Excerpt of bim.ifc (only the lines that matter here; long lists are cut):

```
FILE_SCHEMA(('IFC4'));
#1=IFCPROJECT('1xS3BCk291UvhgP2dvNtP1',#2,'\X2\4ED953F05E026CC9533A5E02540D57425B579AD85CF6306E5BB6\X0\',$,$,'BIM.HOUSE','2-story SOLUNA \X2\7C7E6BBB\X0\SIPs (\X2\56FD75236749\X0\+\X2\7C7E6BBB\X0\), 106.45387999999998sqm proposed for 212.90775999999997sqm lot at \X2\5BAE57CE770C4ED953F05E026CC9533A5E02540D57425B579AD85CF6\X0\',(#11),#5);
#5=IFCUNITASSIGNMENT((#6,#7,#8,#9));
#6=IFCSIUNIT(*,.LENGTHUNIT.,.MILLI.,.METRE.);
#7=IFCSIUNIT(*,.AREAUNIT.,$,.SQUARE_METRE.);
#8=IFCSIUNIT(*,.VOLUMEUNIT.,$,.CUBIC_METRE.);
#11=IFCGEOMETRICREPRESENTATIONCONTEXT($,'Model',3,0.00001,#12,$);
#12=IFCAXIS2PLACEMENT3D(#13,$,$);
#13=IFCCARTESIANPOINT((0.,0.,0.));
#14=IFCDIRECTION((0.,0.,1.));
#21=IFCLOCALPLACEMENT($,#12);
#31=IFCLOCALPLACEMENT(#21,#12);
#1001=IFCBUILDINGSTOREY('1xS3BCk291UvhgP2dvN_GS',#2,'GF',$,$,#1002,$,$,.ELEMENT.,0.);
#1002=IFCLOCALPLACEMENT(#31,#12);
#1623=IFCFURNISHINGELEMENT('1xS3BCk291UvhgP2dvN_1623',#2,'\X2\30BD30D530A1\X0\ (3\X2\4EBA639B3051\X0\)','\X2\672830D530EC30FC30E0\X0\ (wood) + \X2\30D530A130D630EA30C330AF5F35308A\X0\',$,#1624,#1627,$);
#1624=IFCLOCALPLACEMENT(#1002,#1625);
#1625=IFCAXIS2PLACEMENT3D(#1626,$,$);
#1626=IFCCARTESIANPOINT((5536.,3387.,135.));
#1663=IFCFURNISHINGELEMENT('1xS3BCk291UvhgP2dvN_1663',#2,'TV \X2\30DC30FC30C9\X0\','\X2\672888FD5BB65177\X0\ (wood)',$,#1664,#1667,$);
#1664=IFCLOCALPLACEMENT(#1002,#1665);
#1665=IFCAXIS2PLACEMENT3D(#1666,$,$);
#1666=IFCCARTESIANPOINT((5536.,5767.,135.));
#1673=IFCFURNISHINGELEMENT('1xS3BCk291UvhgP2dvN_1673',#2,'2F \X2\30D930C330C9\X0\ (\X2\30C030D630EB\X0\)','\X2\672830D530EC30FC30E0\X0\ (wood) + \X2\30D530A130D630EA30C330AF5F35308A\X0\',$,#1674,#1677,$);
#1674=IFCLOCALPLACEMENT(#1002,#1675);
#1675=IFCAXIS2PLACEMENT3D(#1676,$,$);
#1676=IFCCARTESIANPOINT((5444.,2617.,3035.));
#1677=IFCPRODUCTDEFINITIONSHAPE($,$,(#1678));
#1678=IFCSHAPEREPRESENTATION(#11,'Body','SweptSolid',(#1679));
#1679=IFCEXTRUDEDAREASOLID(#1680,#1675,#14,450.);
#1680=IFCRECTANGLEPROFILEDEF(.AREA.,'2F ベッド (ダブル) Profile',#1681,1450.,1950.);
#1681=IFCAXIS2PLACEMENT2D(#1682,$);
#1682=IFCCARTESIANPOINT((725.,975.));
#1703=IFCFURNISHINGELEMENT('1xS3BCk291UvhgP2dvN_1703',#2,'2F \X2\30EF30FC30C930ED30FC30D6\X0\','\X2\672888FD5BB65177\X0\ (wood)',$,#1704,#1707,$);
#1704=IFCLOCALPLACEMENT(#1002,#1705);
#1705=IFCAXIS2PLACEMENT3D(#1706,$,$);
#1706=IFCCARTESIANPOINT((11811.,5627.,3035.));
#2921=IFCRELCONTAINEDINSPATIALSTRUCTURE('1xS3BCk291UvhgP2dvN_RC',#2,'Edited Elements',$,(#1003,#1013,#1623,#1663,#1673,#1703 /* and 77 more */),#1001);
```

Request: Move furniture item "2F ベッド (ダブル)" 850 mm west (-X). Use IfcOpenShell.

```python
import ifcopenshell
import ifcopenshell.api.geometry
import ifcopenshell.util.placement
import ifcopenshell.util.unit

model = ifcopenshell.open("bim.ifc")
unit_scale = ifcopenshell.util.unit.calculate_unit_scale(model)

item = model.by_guid("1xS3BCk291UvhgP2dvN_1673")
matrix = ifcopenshell.util.placement.get_local_placement(item.ObjectPlacement)
matrix[0, 3] -= 0.85 / unit_scale
ifcopenshell.api.geometry.edit_object_placement(model, product=item, matrix=matrix, is_si=False)

print(ifcopenshell.util.placement.get_local_placement(item.ObjectPlacement).round(3) + 0.0)

model.write("bim_edited.ifc")
```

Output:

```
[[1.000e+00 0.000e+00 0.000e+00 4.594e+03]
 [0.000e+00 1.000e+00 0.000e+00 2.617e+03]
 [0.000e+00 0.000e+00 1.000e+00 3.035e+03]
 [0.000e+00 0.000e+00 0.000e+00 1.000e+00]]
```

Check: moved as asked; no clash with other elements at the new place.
